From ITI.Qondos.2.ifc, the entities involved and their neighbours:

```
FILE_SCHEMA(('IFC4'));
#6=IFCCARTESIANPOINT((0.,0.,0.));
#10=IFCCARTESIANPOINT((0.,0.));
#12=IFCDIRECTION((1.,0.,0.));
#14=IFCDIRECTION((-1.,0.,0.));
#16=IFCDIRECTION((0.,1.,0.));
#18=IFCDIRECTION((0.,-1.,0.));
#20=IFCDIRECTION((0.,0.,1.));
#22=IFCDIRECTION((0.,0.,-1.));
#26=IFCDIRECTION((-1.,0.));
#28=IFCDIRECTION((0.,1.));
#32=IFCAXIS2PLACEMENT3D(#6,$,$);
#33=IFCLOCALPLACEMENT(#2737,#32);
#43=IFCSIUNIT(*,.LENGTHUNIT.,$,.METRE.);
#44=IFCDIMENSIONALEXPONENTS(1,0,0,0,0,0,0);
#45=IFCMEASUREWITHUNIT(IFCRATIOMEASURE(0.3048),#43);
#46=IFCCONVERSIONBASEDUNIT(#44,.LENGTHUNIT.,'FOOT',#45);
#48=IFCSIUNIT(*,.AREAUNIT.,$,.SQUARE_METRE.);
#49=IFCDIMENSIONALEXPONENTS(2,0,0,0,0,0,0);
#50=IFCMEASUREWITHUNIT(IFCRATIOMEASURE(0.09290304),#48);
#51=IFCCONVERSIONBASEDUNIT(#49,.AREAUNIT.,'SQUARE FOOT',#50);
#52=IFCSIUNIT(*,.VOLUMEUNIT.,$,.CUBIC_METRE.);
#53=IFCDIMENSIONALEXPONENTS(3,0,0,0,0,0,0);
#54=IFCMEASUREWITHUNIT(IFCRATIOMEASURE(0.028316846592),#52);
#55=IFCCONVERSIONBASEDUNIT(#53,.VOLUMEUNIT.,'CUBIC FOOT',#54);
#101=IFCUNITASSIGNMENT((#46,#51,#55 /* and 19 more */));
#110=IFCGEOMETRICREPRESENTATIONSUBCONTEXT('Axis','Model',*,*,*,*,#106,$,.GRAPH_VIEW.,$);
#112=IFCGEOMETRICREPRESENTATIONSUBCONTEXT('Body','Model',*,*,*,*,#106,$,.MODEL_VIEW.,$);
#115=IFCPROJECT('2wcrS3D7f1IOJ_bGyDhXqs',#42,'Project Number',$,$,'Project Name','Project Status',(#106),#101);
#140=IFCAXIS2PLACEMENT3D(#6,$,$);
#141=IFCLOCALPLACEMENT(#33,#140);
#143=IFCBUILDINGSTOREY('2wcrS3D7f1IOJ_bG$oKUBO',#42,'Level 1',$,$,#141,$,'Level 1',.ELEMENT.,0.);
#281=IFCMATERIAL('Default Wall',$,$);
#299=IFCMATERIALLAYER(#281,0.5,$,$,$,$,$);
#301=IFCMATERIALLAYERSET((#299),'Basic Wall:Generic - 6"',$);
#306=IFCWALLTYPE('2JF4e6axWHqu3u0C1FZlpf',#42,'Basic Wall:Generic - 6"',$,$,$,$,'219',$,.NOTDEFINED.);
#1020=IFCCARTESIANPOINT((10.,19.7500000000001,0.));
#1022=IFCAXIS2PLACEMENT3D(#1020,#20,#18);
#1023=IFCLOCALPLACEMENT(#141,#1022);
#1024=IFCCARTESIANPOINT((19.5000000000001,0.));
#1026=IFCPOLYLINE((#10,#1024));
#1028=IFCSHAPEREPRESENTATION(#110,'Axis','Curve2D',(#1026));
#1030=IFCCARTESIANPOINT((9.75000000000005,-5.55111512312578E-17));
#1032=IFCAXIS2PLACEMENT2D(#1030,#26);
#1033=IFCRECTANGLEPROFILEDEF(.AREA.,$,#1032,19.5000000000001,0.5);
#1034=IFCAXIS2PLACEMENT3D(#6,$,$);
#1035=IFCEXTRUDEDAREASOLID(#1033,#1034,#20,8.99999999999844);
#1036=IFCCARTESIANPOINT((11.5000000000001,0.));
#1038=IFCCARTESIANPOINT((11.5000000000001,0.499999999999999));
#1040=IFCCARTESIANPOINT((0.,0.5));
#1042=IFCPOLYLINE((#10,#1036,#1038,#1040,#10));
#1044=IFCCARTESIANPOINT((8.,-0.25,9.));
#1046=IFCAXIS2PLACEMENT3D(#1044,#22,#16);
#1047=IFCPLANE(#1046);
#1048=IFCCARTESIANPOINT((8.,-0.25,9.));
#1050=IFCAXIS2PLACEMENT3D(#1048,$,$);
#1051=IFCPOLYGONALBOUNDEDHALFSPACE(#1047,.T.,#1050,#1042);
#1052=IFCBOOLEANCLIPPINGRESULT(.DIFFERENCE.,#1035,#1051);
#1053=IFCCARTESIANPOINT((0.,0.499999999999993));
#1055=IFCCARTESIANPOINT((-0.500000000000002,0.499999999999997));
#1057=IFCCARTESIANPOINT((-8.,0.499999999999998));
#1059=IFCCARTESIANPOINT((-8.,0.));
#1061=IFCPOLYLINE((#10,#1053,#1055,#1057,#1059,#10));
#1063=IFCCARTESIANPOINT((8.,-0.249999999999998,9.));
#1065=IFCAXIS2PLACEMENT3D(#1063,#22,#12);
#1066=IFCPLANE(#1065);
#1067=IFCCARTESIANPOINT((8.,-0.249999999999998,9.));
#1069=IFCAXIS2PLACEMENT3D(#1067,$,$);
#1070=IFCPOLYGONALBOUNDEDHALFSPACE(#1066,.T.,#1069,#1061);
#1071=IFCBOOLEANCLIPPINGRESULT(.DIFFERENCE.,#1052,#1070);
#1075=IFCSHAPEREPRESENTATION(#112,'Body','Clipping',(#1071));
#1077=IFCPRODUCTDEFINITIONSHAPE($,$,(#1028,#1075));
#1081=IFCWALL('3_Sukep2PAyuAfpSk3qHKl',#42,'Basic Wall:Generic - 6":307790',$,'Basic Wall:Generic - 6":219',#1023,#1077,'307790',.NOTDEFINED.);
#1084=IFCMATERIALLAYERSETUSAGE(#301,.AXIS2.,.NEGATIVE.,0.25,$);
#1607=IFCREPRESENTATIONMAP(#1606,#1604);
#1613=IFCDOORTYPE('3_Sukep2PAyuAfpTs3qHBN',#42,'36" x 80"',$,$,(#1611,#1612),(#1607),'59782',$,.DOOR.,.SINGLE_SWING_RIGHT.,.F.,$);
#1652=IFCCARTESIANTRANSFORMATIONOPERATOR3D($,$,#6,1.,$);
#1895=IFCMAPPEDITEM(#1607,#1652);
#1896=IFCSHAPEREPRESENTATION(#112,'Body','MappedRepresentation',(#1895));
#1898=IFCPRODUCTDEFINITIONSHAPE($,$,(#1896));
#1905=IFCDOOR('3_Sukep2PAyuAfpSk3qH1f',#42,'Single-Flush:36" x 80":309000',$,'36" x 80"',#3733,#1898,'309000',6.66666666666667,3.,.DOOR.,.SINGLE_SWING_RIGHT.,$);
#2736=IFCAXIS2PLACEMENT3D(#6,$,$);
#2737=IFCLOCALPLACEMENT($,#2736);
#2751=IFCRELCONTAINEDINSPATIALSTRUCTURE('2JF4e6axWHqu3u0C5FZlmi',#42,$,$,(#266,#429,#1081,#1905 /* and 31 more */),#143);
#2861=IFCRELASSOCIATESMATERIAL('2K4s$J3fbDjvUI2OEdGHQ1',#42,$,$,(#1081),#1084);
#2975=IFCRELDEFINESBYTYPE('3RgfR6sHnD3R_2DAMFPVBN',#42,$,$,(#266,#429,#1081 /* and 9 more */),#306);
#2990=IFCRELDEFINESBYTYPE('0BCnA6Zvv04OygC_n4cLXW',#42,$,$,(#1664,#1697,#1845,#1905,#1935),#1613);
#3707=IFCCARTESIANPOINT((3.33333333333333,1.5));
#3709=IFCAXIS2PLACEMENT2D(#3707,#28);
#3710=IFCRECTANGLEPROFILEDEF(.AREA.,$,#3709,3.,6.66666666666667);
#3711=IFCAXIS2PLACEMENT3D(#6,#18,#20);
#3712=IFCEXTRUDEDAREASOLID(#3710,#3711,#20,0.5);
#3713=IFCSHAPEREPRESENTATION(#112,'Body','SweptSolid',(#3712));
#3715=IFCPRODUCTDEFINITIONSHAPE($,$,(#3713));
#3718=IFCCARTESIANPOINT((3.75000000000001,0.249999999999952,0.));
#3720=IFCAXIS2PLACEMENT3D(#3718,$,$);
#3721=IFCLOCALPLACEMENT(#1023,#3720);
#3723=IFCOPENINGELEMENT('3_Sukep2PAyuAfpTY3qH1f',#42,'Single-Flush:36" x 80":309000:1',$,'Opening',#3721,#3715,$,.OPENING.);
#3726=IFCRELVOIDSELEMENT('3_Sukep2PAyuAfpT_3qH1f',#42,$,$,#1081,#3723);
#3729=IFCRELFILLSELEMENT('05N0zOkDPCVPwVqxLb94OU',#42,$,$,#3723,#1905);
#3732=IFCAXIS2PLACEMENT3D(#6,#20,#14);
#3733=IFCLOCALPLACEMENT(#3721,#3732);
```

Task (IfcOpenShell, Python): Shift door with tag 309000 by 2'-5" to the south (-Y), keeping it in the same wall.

```python
import ifcopenshell
import ifcopenshell.api.geometry
import ifcopenshell.util.placement
import ifcopenshell.util.unit

model = ifcopenshell.open("ITI.Qondos.2.ifc")
unit_scale = ifcopenshell.util.unit.calculate_unit_scale(model)

door = model.by_guid("3_Sukep2PAyuAfpSk3qH1f")
opening = door.FillsVoids[0].RelatingOpeningElement
wall = opening.VoidsElements[0].RelatingBuildingElement

wall_matrix = ifcopenshell.util.placement.get_local_placement(wall.ObjectPlacement)
shift = wall_matrix[:3, 0] * 29 * 0.0254 / unit_scale
before = ifcopenshell.util.placement.get_local_placement(door.ObjectPlacement)[:3, 3].copy()

# The door is placed relative to its opening, so it follows when the opening moves.
matrix = ifcopenshell.util.placement.get_local_placement(opening.ObjectPlacement)
matrix[:3, 3] += shift
ifcopenshell.api.geometry.edit_object_placement(
    model, product=opening, matrix=matrix, is_si=False, should_transform_children=True
)

after = ifcopenshell.util.placement.get_local_placement(door.ObjectPlacement)[:3, 3]
print("door moved by", (after - before).round(3) + 0.0)

model.write("ITI.Qondos.2_rev.ifc")
```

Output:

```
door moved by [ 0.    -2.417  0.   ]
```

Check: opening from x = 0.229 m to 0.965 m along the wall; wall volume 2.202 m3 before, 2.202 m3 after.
